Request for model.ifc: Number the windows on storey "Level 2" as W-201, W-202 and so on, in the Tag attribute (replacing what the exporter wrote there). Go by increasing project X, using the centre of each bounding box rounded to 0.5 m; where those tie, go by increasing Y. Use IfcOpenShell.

First a look at what the model holds.

```python
import ifcopenshell
import ifcopenshell.util.element
import ifcopenshell.util.placement

model = ifcopenshell.open("model.ifc")
print(model.schema)
storey = next(s for s in model.by_type("IfcBuildingStorey") if s.Name == "Level 2")
windows = [e for e in ifcopenshell.util.element.get_decomposition(storey) if e.is_a("IfcWindow")]
for e in sorted(windows, key=lambda e: e.id()):
    origin = ifcopenshell.util.placement.get_local_placement(e.ObjectPlacement)[:3, 3]
    print(e.id(), e.Tag, e.Name, origin.round(2) + 0.0, sep=" | ")
```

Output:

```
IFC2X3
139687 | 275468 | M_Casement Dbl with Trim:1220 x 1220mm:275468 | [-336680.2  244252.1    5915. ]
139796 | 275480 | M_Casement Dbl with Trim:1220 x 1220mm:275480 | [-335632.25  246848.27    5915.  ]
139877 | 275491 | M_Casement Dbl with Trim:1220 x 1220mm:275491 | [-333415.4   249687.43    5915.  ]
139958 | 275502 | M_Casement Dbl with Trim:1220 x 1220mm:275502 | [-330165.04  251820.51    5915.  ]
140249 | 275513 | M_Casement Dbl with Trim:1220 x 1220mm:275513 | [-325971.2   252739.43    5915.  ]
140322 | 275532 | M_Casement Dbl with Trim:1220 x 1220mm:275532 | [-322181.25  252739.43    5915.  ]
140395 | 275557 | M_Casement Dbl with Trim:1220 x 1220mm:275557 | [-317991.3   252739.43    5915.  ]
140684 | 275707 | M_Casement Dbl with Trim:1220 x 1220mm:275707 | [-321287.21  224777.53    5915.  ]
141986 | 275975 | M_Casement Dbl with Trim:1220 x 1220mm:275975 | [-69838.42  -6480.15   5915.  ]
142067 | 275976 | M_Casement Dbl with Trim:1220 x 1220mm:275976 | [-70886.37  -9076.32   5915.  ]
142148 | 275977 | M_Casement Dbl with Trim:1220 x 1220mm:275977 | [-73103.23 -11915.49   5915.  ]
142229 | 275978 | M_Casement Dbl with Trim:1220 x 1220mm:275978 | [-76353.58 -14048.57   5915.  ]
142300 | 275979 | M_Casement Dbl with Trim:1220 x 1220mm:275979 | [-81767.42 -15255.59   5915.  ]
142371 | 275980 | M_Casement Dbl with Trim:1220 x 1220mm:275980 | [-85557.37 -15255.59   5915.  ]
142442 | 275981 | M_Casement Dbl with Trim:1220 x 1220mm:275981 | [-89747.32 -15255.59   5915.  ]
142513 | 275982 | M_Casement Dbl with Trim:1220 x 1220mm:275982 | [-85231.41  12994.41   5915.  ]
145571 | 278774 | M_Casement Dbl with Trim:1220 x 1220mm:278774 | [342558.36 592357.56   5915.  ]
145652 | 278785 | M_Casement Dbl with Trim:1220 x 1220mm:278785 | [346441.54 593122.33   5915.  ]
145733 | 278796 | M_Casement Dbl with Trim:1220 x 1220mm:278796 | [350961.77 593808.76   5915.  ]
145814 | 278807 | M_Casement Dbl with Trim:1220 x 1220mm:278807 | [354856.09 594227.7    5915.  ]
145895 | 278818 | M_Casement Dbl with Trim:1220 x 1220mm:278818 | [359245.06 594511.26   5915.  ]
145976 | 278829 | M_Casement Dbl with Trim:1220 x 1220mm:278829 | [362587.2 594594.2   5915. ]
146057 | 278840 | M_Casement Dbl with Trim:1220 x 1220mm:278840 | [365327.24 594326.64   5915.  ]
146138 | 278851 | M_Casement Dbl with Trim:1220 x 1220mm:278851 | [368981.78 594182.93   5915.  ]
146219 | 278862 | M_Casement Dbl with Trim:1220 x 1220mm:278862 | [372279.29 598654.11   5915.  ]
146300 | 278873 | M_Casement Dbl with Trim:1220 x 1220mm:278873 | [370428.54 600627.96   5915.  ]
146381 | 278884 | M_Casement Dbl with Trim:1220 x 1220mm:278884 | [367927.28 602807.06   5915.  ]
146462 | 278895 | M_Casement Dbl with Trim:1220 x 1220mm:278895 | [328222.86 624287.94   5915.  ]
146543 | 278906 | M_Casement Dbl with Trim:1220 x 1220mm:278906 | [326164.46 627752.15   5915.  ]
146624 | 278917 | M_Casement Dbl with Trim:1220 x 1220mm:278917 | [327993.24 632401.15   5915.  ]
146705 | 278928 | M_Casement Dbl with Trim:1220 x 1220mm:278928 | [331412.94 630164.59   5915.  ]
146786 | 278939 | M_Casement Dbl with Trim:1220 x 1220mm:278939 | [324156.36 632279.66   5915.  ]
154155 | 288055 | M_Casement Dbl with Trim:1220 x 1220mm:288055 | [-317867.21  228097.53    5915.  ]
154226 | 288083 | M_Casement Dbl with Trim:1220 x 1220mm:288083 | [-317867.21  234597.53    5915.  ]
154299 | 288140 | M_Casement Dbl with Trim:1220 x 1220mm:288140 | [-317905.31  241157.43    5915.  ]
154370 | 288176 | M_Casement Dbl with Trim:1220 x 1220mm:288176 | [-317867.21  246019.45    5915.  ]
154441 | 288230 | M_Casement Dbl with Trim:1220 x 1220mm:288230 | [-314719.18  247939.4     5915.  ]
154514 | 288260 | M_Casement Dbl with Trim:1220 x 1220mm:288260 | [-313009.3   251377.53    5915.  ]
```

```python
import ifcopenshell
import ifcopenshell.geom
import ifcopenshell.util.element
import ifcopenshell.util.shape

model = ifcopenshell.open("model.ifc")
settings = ifcopenshell.geom.settings()
settings.set("use-world-coords", True)


def centre(element):
    shape = ifcopenshell.geom.create_shape(settings, element)
    return ifcopenshell.util.shape.get_bbox_centroid(shape.geometry)


storey = next(s for s in model.by_type("IfcBuildingStorey") if s.Name == "Level 2")
windows = [e for e in ifcopenshell.util.element.get_decomposition(storey) if e.is_a("IfcWindow")]

# Insertion points can sit at a corner or the storey origin, so sort by the geometry (in metres).
centres = {e: centre(e) for e in windows}
windows.sort(key=lambda e: (round(centres[e][0] / 0.5), centres[e][1]))

for i, e in enumerate(windows, start=1):
    number = f"W-2{i:02d}"
    e.Tag = number
    print(e.id(), number)

model.write("model-out.ifc")
```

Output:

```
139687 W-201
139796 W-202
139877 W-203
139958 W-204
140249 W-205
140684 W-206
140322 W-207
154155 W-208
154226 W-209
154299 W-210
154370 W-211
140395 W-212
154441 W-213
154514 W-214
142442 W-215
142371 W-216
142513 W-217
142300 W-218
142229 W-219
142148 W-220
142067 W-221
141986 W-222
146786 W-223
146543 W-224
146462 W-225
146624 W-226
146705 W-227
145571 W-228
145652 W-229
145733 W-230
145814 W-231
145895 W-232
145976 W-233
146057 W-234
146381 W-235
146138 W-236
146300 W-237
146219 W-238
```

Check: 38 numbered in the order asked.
